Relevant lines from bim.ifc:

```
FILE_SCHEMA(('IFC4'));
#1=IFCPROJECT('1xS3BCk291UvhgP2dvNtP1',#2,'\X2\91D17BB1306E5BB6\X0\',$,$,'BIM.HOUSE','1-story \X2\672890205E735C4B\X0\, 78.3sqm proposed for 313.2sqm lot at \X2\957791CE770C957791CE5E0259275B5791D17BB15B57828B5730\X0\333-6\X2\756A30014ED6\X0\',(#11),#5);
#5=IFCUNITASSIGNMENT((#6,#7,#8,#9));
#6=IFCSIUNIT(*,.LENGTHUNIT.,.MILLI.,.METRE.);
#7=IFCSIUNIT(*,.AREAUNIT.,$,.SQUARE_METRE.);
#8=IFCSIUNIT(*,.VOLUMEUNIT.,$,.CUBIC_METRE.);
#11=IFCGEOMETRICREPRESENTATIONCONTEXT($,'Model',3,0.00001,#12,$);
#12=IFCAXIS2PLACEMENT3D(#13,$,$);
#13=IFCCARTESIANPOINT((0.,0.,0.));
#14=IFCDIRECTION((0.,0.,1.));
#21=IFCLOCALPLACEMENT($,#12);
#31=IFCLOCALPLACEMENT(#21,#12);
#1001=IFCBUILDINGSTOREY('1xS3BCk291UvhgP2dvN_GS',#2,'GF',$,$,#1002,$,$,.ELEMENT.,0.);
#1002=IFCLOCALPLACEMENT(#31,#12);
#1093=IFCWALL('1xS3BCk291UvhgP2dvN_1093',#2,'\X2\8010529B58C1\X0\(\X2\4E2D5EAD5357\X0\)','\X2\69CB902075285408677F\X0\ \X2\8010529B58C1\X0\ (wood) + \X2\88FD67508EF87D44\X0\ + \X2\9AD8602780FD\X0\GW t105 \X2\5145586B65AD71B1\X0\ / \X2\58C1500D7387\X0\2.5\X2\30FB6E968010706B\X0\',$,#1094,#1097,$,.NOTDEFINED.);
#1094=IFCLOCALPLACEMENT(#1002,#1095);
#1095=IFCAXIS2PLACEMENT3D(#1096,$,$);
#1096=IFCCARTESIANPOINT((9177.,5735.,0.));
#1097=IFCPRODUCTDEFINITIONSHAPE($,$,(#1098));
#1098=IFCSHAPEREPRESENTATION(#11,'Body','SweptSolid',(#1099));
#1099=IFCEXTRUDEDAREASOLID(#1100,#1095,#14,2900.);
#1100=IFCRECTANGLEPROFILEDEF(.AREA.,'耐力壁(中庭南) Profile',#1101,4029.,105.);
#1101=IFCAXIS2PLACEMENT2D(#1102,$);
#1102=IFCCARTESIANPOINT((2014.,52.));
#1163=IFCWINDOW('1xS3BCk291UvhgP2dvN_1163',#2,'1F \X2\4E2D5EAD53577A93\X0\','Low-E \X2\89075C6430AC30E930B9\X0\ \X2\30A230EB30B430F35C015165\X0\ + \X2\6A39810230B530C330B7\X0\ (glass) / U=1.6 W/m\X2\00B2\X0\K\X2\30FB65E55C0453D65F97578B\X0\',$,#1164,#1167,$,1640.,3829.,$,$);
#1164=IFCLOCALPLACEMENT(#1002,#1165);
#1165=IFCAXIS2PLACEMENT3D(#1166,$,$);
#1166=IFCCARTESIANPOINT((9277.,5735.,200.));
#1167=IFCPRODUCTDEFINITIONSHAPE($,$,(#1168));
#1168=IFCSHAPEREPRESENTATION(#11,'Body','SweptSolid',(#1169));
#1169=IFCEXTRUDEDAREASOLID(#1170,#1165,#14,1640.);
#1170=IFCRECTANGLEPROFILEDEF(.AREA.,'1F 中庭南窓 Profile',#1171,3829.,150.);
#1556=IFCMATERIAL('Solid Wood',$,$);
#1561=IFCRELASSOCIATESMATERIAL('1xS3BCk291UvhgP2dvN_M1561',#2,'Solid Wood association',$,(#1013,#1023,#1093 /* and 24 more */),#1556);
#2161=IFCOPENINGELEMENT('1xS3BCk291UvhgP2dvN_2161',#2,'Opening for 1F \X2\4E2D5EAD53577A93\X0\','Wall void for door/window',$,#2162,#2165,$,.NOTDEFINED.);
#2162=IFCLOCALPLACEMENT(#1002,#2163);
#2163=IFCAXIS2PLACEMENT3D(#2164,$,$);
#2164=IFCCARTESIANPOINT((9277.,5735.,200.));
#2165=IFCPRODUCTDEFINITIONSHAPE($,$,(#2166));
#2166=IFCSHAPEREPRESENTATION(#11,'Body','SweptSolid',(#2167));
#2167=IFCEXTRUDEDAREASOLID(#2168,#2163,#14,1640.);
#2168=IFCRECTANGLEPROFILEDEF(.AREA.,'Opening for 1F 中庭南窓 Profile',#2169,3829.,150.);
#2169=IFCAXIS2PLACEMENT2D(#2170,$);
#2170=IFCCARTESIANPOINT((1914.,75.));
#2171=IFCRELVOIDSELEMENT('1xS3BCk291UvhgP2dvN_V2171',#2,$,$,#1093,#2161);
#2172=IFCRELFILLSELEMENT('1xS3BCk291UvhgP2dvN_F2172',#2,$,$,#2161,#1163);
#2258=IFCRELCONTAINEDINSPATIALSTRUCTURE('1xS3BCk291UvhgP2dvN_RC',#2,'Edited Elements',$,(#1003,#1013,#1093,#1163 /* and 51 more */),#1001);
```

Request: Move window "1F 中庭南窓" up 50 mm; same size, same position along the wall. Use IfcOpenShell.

```python
import numpy as np
import ifcopenshell
import ifcopenshell.api.geometry
import ifcopenshell.util.placement
import ifcopenshell.util.unit

model = ifcopenshell.open("bim.ifc")
unit_scale = ifcopenshell.util.unit.calculate_unit_scale(model)

window = model.by_id(1163)
opening = window.FillsVoids[0].RelatingOpeningElement
dz = 0.05 / unit_scale

shift = np.array([0.0, 0.0, dz])
# The window is not placed relative to its opening, so move both.
for product in (opening, window):
    matrix = ifcopenshell.util.placement.get_local_placement(product.ObjectPlacement)
    matrix[:3, 3] += shift
    ifcopenshell.api.geometry.edit_object_placement(model, product=product, matrix=matrix, is_si=False)

print(f"moved by {dz * unit_scale:+.3f} m")

model.write("bim-out.ifc")
```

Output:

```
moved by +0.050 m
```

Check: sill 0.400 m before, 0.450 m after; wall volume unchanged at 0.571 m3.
